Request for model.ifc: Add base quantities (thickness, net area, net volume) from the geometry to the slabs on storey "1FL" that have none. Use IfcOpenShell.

First a look at what the model holds.

```python
import ifcopenshell
import ifcopenshell.util.element
import ifcopenshell.util.unit

model = ifcopenshell.open("model.ifc")
print(model.schema)
for unit_type in ("LENGTHUNIT", "AREAUNIT", "VOLUMEUNIT"):
    print(unit_type, ifcopenshell.util.unit.calculate_unit_scale(model, unit_type))
storey = next(s for s in model.by_type("IfcBuildingStorey") if s.Name == "1FL")
slabs = [e for e in ifcopenshell.util.element.get_decomposition(storey) if e.is_a("IfcSlab")]
for e in sorted(slabs, key=lambda e: e.id()):
    print(e.id(), e.is_a(), e.Name, list(ifcopenshell.util.element.get_psets(e, qtos_only=True)), sep=" | ")
```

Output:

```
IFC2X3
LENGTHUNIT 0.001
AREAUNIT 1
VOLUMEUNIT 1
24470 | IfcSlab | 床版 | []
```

```python
import ifcopenshell
import ifcopenshell.api.pset
import ifcopenshell.geom
import ifcopenshell.util.element
import ifcopenshell.util.shape
import ifcopenshell.util.unit

model = ifcopenshell.open("model.ifc")
unit_scale = ifcopenshell.util.unit.calculate_unit_scale(model)
area_scale = ifcopenshell.util.unit.calculate_unit_scale(model, "AREAUNIT")
volume_scale = ifcopenshell.util.unit.calculate_unit_scale(model, "VOLUMEUNIT")
settings = ifcopenshell.geom.settings()

storey = next(s for s in model.by_type("IfcBuildingStorey") if s.Name == "1FL")
slabs = [e for e in ifcopenshell.util.element.get_decomposition(storey) if e.is_a("IfcSlab")]

for e in sorted(slabs, key=lambda e: e.id()):
    if ifcopenshell.util.element.get_psets(e, qtos_only=True, should_inherit=False):
        continue
    # Geometry comes back in metres, in the element's own axes.
    shape = ifcopenshell.geom.create_shape(settings, e)
    values = {
        "Width": ifcopenshell.util.shape.get_z(shape.geometry) / unit_scale,
        "NetArea": ifcopenshell.util.shape.get_footprint_area(shape.geometry) / area_scale,
        "NetVolume": ifcopenshell.util.shape.get_volume(shape.geometry) / volume_scale,
    }
    qto = ifcopenshell.api.pset.add_qto(model, product=e, name="BaseQuantities")
    ifcopenshell.api.pset.edit_qto(model, qto=qto, properties=values)
    print(e.id(), {k: round(v, 3) for k, v in values.items()})

model.write("model_v2.ifc")
```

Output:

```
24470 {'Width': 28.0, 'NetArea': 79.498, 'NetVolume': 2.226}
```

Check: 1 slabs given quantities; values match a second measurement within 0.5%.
